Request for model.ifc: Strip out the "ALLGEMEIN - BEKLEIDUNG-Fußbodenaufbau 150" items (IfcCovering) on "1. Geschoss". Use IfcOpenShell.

First a look at what the model holds.

```python
import ifcopenshell
import ifcopenshell.util.element

model = ifcopenshell.open("model.ifc")
print(model.schema)
storey = next(s for s in model.by_type("IfcBuildingStorey") if s.Name == "1. Geschoss")
coverings = [e for e in ifcopenshell.util.element.get_decomposition(storey) if e.is_a("IfcCovering")]
seen = {}
for e in coverings:
    element_type = ifcopenshell.util.element.get_type(e)
    name = element_type.Name if element_type not in (None, e) else None
    seen[name] = seen.get(name, 0) + 1
for name, count in sorted(seen.items(), key=str):
    print(count, "x", name)
```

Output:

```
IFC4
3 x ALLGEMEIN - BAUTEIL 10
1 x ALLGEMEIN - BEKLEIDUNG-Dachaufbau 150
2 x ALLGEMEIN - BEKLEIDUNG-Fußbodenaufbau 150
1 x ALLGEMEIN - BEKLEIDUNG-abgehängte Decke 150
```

```python
import ifcopenshell
import ifcopenshell.api.root
import ifcopenshell.util.element

model = ifcopenshell.open("model.ifc")

storey = next(s for s in model.by_type("IfcBuildingStorey") if s.Name == "1. Geschoss")
coverings = [e for e in ifcopenshell.util.element.get_decomposition(storey) if e.is_a("IfcCovering")]
targets = [e for e in coverings if (t := ifcopenshell.util.element.get_type(e)) not in (None, e) and t.Name == "ALLGEMEIN - BEKLEIDUNG-Fußbodenaufbau 150"]

for e in targets:
    ifcopenshell.api.root.remove_product(model, product=e)
print(len(targets), "removed")

model.write("model_v2.ifc")
```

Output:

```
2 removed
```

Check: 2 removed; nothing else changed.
